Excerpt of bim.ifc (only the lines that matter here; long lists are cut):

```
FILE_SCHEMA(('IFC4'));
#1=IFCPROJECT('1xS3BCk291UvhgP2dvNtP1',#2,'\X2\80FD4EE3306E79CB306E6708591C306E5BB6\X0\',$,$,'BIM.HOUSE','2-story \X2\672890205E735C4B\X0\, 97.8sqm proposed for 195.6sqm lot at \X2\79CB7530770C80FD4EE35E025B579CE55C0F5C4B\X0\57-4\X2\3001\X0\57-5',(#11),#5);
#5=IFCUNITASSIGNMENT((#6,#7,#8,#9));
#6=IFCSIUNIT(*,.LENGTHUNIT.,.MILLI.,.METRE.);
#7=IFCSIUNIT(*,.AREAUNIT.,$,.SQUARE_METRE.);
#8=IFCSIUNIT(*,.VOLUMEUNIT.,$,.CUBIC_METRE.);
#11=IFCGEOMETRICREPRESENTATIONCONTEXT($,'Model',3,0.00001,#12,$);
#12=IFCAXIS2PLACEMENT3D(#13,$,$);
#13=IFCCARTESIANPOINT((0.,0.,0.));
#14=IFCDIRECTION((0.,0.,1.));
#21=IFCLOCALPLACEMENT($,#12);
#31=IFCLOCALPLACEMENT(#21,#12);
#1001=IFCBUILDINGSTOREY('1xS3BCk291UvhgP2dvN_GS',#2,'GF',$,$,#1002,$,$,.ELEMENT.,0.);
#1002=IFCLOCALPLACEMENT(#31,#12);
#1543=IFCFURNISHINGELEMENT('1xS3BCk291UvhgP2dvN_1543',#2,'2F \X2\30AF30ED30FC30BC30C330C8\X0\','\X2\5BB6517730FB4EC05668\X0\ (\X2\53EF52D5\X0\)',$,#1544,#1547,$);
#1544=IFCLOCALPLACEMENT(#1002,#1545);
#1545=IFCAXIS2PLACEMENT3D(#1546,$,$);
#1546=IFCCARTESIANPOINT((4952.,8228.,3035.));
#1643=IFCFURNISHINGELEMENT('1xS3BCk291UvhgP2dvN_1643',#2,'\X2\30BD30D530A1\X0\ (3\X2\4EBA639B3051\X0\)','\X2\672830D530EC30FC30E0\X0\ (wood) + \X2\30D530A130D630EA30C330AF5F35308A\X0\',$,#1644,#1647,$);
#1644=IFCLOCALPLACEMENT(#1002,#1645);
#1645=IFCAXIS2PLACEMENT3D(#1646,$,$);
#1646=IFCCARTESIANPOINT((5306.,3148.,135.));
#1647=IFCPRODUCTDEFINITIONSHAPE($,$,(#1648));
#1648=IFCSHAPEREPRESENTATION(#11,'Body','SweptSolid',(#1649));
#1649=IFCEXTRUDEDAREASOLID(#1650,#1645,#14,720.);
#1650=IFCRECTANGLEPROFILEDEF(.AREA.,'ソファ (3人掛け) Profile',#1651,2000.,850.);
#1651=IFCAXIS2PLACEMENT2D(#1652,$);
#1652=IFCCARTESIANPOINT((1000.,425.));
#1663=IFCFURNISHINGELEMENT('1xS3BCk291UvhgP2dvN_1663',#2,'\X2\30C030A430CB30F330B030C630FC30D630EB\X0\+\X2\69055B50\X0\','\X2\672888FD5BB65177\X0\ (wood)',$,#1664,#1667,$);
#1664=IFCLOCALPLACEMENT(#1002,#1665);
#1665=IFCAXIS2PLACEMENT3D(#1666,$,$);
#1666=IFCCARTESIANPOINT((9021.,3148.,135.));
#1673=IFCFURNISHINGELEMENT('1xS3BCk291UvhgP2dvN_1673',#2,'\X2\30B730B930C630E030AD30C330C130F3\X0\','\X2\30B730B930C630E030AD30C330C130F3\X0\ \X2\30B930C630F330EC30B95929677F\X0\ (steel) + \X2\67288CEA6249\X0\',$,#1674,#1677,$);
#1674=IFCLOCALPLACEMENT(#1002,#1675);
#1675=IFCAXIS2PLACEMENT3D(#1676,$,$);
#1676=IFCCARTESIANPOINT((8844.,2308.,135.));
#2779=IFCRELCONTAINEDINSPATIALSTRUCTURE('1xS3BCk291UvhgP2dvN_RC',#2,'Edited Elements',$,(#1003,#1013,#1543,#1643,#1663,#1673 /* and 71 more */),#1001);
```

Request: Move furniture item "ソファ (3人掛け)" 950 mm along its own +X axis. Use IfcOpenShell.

```python
import ifcopenshell
import ifcopenshell.api.geometry
import ifcopenshell.util.placement

model = ifcopenshell.open("bim.ifc")

item = model.by_id(1643)
matrix = ifcopenshell.util.placement.get_local_placement(item.ObjectPlacement)
matrix[:3, 3] += matrix[:3, 0] * 950.0
ifcopenshell.api.geometry.edit_object_placement(model, product=item, matrix=matrix, is_si=False)

print(ifcopenshell.util.placement.get_local_placement(item.ObjectPlacement).round(3) + 0.0)

model.write("bim_v2.ifc")
```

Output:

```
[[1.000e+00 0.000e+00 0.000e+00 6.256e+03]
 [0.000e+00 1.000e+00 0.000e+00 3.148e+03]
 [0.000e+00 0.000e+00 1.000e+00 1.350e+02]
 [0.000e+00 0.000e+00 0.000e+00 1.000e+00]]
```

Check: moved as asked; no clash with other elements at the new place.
